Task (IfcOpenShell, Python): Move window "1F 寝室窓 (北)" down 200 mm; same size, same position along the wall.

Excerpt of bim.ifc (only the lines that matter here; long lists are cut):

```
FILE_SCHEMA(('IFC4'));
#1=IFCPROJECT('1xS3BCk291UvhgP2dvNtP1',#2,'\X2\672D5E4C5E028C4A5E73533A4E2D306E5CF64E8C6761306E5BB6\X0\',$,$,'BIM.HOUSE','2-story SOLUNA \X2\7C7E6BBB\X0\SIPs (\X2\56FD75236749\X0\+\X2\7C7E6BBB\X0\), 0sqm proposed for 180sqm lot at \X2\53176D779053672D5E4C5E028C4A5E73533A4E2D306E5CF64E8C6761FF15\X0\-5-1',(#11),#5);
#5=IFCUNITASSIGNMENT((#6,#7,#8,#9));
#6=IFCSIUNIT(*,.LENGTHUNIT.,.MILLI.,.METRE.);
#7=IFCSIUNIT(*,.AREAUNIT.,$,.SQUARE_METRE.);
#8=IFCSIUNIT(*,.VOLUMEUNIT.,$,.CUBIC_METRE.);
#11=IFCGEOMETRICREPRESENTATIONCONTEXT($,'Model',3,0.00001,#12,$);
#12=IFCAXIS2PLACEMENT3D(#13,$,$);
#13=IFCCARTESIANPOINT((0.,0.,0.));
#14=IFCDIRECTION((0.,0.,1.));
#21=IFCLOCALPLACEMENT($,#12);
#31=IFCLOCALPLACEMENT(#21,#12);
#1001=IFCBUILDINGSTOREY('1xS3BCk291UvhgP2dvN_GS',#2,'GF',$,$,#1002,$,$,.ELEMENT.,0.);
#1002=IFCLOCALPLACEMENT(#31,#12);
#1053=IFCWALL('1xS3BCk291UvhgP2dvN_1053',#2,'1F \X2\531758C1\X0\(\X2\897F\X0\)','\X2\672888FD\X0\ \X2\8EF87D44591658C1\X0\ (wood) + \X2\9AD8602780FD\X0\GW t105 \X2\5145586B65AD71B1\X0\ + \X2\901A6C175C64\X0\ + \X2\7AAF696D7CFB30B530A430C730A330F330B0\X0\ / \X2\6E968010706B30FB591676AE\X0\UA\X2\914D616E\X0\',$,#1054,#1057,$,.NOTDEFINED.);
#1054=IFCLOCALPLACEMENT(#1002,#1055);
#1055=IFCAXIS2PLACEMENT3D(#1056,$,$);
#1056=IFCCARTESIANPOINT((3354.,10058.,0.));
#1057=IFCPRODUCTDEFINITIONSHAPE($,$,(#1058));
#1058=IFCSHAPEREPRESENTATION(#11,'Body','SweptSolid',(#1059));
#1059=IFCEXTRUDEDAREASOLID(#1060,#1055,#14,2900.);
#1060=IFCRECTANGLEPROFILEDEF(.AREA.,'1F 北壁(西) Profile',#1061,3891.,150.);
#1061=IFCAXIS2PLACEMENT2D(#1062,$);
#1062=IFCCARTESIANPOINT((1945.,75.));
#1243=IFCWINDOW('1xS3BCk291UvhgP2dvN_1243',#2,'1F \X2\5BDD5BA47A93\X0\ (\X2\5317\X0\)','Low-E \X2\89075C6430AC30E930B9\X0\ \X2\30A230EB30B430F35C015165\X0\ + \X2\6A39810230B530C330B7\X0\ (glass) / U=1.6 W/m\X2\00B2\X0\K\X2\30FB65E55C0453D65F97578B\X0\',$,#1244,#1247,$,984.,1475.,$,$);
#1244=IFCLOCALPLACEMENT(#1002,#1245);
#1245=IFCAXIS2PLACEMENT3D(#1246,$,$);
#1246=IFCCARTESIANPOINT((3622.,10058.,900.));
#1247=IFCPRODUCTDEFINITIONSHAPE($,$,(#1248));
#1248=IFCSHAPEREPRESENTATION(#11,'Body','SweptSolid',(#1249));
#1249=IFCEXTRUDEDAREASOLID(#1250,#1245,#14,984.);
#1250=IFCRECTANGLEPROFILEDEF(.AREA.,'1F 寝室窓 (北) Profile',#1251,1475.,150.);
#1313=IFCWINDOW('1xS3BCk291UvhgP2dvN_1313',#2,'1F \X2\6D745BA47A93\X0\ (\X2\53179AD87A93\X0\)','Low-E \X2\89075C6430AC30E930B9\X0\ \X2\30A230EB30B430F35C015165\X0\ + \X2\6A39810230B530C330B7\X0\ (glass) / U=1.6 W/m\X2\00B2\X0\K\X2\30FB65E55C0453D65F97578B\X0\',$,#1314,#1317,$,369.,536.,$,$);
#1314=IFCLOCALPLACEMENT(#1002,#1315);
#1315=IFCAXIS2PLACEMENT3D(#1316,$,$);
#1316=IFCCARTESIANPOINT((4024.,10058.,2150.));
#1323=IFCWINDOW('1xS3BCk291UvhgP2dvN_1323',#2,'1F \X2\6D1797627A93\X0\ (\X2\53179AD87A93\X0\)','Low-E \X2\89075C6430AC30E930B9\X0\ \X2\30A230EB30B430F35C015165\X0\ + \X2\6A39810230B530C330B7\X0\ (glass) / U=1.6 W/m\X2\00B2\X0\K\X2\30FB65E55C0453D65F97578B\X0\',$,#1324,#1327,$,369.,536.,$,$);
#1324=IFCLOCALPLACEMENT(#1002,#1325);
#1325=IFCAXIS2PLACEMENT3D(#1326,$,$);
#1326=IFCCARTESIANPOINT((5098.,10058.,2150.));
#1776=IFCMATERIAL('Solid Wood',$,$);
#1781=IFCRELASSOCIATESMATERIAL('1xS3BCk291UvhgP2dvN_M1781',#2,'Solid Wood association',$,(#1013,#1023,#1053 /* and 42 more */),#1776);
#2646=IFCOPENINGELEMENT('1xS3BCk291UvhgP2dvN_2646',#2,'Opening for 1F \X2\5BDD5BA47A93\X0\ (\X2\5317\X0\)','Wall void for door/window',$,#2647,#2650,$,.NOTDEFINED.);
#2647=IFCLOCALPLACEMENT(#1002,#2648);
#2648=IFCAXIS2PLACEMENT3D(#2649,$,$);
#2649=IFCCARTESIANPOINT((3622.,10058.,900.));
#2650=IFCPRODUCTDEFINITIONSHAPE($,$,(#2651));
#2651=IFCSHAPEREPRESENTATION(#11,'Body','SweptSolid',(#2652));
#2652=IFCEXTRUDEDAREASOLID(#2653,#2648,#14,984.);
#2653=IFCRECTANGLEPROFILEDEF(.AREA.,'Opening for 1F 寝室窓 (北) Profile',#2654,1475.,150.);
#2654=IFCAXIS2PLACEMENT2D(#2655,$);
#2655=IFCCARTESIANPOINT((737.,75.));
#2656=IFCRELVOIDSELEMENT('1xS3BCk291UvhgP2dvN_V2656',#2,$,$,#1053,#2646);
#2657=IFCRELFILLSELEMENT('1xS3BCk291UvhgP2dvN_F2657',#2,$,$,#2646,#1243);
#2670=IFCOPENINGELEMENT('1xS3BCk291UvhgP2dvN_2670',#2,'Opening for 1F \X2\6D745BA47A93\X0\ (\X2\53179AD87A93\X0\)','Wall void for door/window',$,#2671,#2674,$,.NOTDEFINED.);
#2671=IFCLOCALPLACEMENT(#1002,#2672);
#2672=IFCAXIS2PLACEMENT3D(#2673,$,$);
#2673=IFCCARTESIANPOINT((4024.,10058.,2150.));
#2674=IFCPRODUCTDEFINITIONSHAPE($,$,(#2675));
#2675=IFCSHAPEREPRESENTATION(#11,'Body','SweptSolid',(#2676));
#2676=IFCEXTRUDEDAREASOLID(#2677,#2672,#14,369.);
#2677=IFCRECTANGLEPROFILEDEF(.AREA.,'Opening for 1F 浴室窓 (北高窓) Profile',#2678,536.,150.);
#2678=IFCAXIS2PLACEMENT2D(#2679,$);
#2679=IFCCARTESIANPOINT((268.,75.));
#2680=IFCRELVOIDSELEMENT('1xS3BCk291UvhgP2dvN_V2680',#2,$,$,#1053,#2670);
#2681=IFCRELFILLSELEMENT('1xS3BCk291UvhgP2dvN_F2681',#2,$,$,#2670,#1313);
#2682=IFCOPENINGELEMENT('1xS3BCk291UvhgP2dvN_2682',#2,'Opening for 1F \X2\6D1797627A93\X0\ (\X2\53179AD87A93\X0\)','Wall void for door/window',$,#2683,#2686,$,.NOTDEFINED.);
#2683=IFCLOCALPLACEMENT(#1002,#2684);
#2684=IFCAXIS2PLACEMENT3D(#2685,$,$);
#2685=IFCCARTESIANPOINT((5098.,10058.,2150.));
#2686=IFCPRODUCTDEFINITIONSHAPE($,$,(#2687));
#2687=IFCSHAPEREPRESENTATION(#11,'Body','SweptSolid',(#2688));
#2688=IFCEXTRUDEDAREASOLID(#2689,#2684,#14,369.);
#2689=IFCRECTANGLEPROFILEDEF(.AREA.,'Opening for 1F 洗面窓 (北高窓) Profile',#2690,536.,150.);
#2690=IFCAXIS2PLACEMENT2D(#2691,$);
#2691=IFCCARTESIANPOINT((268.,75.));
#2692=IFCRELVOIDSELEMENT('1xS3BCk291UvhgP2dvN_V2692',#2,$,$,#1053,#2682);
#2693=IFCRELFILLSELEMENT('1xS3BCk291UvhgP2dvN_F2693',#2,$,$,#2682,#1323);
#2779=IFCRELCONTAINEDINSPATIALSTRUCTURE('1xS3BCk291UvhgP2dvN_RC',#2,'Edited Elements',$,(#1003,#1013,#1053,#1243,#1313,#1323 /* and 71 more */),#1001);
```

```python
import numpy as np
import ifcopenshell
import ifcopenshell.api.geometry
import ifcopenshell.util.placement
import ifcopenshell.util.unit

model = ifcopenshell.open("bim.ifc")
unit_scale = ifcopenshell.util.unit.calculate_unit_scale(model)

window = model.by_id(1243)
opening = window.FillsVoids[0].RelatingOpeningElement
dz = -0.2 / unit_scale

shift = np.array([0.0, 0.0, dz])
# The window is not placed relative to its opening, so move both.
for product in (opening, window):
    matrix = ifcopenshell.util.placement.get_local_placement(product.ObjectPlacement)
    matrix[:3, 3] += shift
    ifcopenshell.api.geometry.edit_object_placement(model, product=product, matrix=matrix, is_si=False)

print(f"moved by {dz * unit_scale:+.3f} m")

model.write("bim_edited.ifc")
```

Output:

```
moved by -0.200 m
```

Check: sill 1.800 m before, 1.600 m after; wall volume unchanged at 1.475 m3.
